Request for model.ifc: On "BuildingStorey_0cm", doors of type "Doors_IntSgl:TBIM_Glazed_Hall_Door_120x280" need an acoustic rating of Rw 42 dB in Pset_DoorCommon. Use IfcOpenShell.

First a look at what the model holds.

```python
import ifcopenshell
import ifcopenshell.util.element

model = ifcopenshell.open("model.ifc")
print(model.schema)
storey = next(s for s in model.by_type("IfcBuildingStorey") if s.Name == "BuildingStorey_0cm")
doors = [e for e in ifcopenshell.util.element.get_decomposition(storey) if e.is_a("IfcDoor")]
seen = {}
for e in doors:
    element_type = ifcopenshell.util.element.get_type(e)
    key = (element_type.Name if element_type != e and element_type else None, ifcopenshell.util.element.get_pset(e, "Pset_DoorCommon", "AcousticRating"))
    seen[key] = seen.get(key, 0) + 1
for (name, value), count in sorted(seen.items(), key=str):
    print(count, "x", name, "|", value)
```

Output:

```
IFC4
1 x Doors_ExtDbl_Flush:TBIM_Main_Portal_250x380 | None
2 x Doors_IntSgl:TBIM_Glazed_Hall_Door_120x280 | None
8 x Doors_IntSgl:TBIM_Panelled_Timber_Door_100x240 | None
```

```python
import ifcopenshell
import ifcopenshell.api.pset
import ifcopenshell.util.element

model = ifcopenshell.open("model.ifc")

storey = next(s for s in model.by_type("IfcBuildingStorey") if s.Name == "BuildingStorey_0cm")
doors = [e for e in ifcopenshell.util.element.get_decomposition(storey) if e.is_a("IfcDoor")]

count = 0
for e in doors:
    element_type = ifcopenshell.util.element.get_type(e)
    if element_type in (None, e) or element_type.Name != "Doors_IntSgl:TBIM_Glazed_Hall_Door_120x280":
        continue
    # add_pset returns the element's existing set when there is one.
    pset = ifcopenshell.api.pset.add_pset(model, product=e, name="Pset_DoorCommon")
    ifcopenshell.api.pset.edit_pset(model, pset=pset, properties={"AcousticRating": "Rw 42 dB"})
    count += 1

print(count, "doors updated")

model.write("model_rev.ifc")
```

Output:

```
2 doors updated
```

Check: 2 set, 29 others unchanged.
